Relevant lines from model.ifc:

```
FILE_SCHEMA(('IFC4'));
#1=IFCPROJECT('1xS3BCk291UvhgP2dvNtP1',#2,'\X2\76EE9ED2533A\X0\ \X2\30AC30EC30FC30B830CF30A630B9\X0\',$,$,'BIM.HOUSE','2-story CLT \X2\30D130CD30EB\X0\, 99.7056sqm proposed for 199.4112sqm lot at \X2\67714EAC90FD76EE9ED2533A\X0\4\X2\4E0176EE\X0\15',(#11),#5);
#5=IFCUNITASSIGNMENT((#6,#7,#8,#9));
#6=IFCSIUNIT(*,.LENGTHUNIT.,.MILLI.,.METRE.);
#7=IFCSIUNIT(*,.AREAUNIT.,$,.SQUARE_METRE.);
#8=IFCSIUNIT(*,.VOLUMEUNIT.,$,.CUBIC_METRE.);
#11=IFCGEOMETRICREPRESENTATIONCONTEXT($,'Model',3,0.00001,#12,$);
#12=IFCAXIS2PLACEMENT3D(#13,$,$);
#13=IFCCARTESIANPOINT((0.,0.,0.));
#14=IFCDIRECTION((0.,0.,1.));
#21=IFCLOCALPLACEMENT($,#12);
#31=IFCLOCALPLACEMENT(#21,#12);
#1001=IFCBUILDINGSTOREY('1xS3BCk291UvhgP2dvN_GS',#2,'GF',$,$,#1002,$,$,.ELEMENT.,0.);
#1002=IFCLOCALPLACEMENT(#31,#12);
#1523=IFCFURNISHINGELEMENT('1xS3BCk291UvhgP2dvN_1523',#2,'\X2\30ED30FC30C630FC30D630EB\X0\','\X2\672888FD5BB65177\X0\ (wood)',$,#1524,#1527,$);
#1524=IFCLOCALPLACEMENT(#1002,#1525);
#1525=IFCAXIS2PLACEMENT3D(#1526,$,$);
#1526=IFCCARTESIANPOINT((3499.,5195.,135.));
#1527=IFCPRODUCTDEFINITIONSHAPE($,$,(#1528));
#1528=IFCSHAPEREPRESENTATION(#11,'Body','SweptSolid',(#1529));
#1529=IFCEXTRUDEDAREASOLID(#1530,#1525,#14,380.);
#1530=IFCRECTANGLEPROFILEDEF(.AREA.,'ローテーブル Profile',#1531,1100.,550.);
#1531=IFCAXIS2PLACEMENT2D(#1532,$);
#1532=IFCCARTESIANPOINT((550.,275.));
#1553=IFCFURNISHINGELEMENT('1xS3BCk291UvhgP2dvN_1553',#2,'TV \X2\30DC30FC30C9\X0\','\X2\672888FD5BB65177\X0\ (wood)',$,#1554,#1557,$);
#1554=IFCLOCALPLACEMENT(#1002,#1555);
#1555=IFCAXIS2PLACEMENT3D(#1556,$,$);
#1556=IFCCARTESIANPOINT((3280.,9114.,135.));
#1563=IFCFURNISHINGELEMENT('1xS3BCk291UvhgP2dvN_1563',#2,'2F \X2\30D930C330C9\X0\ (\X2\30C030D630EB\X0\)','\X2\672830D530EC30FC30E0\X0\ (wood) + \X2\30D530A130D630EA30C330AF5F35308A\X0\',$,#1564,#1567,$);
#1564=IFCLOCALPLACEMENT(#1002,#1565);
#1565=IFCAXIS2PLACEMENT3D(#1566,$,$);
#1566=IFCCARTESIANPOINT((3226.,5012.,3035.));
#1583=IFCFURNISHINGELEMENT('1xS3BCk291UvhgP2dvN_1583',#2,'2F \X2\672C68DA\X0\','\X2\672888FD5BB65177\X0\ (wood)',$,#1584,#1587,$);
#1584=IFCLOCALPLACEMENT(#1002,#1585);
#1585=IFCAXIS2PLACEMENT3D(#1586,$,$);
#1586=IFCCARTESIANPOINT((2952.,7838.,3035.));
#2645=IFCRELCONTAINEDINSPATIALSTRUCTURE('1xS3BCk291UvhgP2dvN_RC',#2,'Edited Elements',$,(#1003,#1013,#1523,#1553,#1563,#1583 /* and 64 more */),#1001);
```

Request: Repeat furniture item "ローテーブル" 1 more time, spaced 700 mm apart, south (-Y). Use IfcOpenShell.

```python
import numpy as np
import ifcopenshell
import ifcopenshell.api.geometry
import ifcopenshell.api.root
import ifcopenshell.util.element
import ifcopenshell.util.placement
import ifcopenshell.util.unit

model = ifcopenshell.open("model.ifc")
unit_scale = ifcopenshell.util.unit.calculate_unit_scale(model)


def reuse_history(source, copy):
    """copy_class also copies each property set's owner history, people and application; keep the originals."""
    for rel in copy.IsDefinedBy:
        if rel.is_a("IfcRelDefinesByProperties") and (history := rel.RelatingPropertyDefinition.OwnerHistory):
            rel.RelatingPropertyDefinition.OwnerHistory = source.OwnerHistory
            ifcopenshell.util.element.remove_deep2(model, history)


source = model.by_guid("1xS3BCk291UvhgP2dvN_1523")
base = ifcopenshell.util.placement.get_local_placement(source.ObjectPlacement)
step = np.array([0.0, -1.0, 0.0]) * 0.7 / unit_scale

for i in range(1, 2):
    copy = ifcopenshell.api.root.copy_class(model, product=source)
    copy.Representation = ifcopenshell.util.element.copy_deep(
        model, source.Representation, exclude=["IfcGeometricRepresentationContext", "IfcRepresentationMap"]
    )
    reuse_history(source, copy)
    matrix = base.copy()
    matrix[:3, 3] += i * step
    print("added at", matrix[:3, 3].round(3) + 0.0)
    ifcopenshell.api.geometry.edit_object_placement(model, product=copy, matrix=matrix, is_si=False)

model.write("model_rev.ifc")
```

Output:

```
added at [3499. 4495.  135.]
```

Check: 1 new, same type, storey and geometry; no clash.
